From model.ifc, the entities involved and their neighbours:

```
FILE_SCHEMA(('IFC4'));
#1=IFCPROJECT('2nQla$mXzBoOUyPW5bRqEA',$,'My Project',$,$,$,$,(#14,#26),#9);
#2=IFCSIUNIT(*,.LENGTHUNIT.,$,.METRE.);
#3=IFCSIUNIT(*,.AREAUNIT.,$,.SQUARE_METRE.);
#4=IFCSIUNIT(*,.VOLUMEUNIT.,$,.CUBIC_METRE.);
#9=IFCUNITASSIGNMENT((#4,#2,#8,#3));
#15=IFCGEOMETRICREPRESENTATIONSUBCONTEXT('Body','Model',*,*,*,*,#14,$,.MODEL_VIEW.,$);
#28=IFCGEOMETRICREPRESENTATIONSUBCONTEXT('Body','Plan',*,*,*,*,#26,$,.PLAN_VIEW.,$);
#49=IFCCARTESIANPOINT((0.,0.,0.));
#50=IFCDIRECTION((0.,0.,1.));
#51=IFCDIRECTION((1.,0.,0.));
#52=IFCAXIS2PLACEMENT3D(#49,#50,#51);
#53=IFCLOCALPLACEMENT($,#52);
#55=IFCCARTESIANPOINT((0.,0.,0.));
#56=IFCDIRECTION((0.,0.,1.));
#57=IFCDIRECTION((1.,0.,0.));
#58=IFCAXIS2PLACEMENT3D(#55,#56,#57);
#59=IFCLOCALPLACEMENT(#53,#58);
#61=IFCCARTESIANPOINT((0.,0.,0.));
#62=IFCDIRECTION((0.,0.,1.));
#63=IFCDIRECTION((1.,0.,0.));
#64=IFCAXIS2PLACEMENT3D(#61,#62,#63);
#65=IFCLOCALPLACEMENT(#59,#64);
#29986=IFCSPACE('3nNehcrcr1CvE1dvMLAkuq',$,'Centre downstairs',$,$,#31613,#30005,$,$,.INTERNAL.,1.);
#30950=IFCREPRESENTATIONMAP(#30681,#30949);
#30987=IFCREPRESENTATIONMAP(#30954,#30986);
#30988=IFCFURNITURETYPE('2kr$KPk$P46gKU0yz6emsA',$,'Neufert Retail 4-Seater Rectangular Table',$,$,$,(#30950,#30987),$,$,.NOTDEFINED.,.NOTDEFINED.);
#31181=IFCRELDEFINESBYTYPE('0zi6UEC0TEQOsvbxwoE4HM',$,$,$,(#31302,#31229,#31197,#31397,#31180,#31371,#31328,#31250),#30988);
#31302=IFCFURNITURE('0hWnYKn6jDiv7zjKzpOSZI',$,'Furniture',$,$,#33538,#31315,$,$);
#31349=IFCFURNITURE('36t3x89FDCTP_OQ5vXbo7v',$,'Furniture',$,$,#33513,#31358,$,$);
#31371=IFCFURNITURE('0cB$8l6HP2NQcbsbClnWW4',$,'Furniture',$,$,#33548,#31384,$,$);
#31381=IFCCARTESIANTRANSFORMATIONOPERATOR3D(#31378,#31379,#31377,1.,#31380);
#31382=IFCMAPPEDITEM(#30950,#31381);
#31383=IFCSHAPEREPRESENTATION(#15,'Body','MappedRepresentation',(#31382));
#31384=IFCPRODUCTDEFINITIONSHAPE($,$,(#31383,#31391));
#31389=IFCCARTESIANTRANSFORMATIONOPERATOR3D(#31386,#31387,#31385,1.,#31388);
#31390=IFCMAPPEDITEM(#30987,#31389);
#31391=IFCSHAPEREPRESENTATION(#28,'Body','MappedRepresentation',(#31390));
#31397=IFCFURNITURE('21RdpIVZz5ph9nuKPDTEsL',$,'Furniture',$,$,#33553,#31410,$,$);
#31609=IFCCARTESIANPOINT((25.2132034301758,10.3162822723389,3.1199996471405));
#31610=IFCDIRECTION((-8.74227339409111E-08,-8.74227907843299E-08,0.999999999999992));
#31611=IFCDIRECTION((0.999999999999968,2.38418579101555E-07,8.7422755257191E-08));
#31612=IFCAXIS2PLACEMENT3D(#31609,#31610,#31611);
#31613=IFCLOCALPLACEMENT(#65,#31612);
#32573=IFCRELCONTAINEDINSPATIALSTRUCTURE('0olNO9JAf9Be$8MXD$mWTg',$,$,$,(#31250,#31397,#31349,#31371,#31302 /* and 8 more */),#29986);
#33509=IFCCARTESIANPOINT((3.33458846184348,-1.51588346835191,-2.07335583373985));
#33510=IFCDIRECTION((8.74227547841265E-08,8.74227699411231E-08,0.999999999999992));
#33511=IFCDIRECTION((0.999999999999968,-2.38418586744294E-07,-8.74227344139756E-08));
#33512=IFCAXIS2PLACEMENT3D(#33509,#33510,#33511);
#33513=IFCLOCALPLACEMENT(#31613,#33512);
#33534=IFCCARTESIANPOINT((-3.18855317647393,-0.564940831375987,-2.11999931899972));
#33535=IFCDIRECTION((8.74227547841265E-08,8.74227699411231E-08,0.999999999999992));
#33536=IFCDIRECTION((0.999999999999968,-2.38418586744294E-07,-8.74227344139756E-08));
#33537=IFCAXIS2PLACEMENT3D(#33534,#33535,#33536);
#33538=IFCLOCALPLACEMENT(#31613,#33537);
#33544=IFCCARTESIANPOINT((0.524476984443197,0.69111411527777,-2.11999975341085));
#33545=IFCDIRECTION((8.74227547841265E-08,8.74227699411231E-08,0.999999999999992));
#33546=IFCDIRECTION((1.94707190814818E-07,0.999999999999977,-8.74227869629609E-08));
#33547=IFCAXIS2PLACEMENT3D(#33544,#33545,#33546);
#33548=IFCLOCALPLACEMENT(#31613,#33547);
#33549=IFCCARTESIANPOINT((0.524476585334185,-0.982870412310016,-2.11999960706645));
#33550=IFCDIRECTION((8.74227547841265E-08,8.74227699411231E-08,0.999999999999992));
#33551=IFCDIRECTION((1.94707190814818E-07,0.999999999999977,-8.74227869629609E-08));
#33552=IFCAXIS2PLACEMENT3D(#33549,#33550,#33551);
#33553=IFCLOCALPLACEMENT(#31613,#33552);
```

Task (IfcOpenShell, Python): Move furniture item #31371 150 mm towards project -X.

```python
import ifcopenshell
import ifcopenshell.api.geometry
import ifcopenshell.util.placement
import ifcopenshell.util.unit

model = ifcopenshell.open("model.ifc")
unit_scale = ifcopenshell.util.unit.calculate_unit_scale(model)

item = model.by_guid("0cB$8l6HP2NQcbsbClnWW4")
matrix = ifcopenshell.util.placement.get_local_placement(item.ObjectPlacement)
matrix[0, 3] -= 0.15 / unit_scale
ifcopenshell.api.geometry.edit_object_placement(model, product=item, matrix=matrix, is_si=False)

print(ifcopenshell.util.placement.get_local_placement(item.ObjectPlacement).round(3) + 0.0)

model.write("model_edited.ifc")
```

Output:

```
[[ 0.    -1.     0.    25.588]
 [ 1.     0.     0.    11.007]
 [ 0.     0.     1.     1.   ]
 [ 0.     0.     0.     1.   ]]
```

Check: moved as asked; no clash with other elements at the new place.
